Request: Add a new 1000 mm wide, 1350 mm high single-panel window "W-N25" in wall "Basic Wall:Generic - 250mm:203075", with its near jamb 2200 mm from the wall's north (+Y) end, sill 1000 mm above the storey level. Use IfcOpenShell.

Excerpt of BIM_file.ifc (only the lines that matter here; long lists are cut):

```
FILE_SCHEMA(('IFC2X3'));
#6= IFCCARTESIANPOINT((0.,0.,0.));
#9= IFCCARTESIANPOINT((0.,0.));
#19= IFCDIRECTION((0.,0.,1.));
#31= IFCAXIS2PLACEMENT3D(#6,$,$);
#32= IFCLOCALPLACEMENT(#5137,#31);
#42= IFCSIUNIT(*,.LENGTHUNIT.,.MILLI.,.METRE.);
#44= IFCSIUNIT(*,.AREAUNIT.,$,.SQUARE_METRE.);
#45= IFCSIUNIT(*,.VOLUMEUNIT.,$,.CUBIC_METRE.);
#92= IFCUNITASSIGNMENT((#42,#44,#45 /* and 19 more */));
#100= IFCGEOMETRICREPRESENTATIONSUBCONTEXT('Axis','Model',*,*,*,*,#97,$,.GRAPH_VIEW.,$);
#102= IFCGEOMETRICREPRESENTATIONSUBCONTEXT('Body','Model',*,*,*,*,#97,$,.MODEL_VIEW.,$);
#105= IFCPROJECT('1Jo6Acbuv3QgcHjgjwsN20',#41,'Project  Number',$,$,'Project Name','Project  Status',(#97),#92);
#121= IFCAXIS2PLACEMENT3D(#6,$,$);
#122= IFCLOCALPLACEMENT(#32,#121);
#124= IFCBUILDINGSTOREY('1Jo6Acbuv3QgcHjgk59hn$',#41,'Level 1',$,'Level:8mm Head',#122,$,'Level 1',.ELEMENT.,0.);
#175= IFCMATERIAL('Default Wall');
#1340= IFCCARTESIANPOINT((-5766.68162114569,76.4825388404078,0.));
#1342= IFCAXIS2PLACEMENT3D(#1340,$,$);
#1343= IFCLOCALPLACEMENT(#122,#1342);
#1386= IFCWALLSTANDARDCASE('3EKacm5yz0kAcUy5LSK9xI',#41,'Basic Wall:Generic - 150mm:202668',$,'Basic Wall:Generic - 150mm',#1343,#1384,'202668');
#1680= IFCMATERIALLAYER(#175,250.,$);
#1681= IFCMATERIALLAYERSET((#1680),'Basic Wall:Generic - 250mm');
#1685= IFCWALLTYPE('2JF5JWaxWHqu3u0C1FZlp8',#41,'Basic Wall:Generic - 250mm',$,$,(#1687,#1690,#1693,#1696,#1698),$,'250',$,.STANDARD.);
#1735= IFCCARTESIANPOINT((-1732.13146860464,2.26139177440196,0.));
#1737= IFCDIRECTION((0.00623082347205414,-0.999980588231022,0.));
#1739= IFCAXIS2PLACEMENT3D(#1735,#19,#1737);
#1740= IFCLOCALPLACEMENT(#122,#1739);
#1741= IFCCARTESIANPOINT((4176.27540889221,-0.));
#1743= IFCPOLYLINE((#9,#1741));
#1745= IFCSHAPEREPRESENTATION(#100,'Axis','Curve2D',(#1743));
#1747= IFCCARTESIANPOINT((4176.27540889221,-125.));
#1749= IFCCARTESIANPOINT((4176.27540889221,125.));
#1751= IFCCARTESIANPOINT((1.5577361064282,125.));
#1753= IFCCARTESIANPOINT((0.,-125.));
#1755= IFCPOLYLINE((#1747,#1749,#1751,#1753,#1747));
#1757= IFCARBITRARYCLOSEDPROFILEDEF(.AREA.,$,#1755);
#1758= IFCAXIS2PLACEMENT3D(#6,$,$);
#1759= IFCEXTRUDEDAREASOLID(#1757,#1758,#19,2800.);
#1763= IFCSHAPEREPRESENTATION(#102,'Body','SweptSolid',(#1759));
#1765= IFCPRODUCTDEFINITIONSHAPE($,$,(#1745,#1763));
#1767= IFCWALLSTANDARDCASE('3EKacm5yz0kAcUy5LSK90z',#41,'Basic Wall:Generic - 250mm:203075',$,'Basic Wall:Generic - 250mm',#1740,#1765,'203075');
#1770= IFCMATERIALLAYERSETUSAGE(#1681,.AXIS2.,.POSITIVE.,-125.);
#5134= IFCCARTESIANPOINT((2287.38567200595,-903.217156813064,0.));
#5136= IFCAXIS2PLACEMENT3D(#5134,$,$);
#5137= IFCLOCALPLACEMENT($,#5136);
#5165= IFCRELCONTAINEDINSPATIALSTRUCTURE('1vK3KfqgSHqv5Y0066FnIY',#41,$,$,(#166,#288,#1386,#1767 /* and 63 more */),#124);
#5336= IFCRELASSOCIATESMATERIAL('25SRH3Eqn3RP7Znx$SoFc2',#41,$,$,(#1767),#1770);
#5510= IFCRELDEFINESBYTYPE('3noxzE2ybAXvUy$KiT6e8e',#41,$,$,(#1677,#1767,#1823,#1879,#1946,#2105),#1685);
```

```python
import numpy as np
import ifcopenshell
import ifcopenshell.api.feature
import ifcopenshell.api.geometry
import ifcopenshell.api.root
import ifcopenshell.api.spatial
import ifcopenshell.api.type
import ifcopenshell.geom
import ifcopenshell.util.element
import ifcopenshell.util.placement
import ifcopenshell.util.representation
import ifcopenshell.util.shape
import ifcopenshell.util.unit

model = ifcopenshell.open("BIM_file.ifc")
unit_scale = ifcopenshell.util.unit.calculate_unit_scale(model)
settings = ifcopenshell.geom.settings()


def volume(element):
    """Net volume in cubic metres, openings subtracted."""
    shape = ifcopenshell.geom.create_shape(settings, element)
    return ifcopenshell.util.shape.get_volume(shape.geometry)


wall = model.by_guid("3EKacm5yz0kAcUy5LSK90z")
storey = ifcopenshell.util.element.get_container(wall, ifc_class="IfcBuildingStorey")
context = ifcopenshell.util.representation.get_context(model, "Model", "Body", "MODEL_VIEW")
before = volume(wall)

width, height, from_end, sill = 1, 1.35, 2.2, 1  # metres

# The wall runs along its own X axis, and the end named is its -X end.
wall_shape = ifcopenshell.geom.create_shape(settings, wall)
x, y, z = ifcopenshell.util.shape.get_vertices(wall_shape.geometry).T
start = x.min() + from_end
face, thickness = float(y.min()), float(y.max() - y.min())
wall_matrix = ifcopenshell.util.placement.get_local_placement(wall.ObjectPlacement)
level = ifcopenshell.util.placement.get_local_placement(storey.ObjectPlacement)[2, 3]


def in_wall(x, y):
    """Placement at x, y metres in the wall's axes, at sill height."""
    matrix = wall_matrix.copy()
    matrix[:, 3] = wall_matrix @ np.array([x / unit_scale, y / unit_scale, 0.0, 1.0])
    matrix[2, 3] = level + sill / unit_scale
    return matrix


# Opening: a box that overshoots both wall faces by 50 mm.
opening = ifcopenshell.api.root.create_entity(model, ifc_class="IfcOpeningElement")
box = ifcopenshell.api.geometry.add_wall_representation(
    model, context=context, length=width, height=height, thickness=thickness + 0.1
)
ifcopenshell.api.geometry.assign_representation(model, product=opening, representation=box)
ifcopenshell.api.geometry.edit_object_placement(model, product=opening, matrix=in_wall(start, face - 0.05), is_si=False)
ifcopenshell.api.feature.add_feature(model, feature=opening, element=wall)

window = ifcopenshell.api.root.create_entity(model, ifc_class="IfcWindow", name="W-N25")
window.OverallWidth, window.OverallHeight = width / unit_scale, height / unit_scale
body = ifcopenshell.api.geometry.add_window_representation(
    model,
    context=context,
    overall_width=window.OverallWidth,
    overall_height=window.OverallHeight,
    partition_type="SINGLE_PANEL",
)
ifcopenshell.api.geometry.assign_representation(model, product=window, representation=body)
ifcopenshell.api.spatial.assign_container(model, products=[window], relating_structure=storey)
fills = ifcopenshell.api.feature.add_filling(model, opening=opening, element=window)
fills.OwnerHistory = window.OwnerHistory  # required in IFC2X3

# IFC2X3 keeps the operation on the window style.
style = ifcopenshell.api.root.create_entity(model, ifc_class="IfcWindowStyle", name="W-N25")
style.OperationType, style.ConstructionType = "SINGLE_PANEL", "NOTDEFINED"
style.ParameterTakesPrecedence = style.Sizeable = False
ifcopenshell.api.type.assign_type(model, related_objects=[window], relating_type=style)

# Centre the window in the wall's thickness.
ifcopenshell.api.geometry.edit_object_placement(model, product=window, matrix=in_wall(start, face), is_si=False)
window_shape = ifcopenshell.geom.create_shape(settings, window)
depth = ifcopenshell.util.shape.get_vertices(window_shape.geometry)[:, 1]
offset = face + thickness / 2 - (depth.min() + depth.max()) / 2
ifcopenshell.api.geometry.edit_object_placement(model, product=window, matrix=in_wall(start, offset), is_si=False)

after = volume(wall)

print(f"wall volume {before:.3f} -> {after:.3f} m3")

model.write("BIM_file_v2.ifc")
```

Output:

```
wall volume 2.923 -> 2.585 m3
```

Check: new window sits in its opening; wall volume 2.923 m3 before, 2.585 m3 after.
